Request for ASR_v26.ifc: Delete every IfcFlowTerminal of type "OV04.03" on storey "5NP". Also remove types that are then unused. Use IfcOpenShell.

First a look at what the model holds.

```python
import ifcopenshell
import ifcopenshell.util.element

model = ifcopenshell.open("ASR_v26.ifc")
print(model.schema)
storey = next(s for s in model.by_type("IfcBuildingStorey") if s.Name == "5NP")
terminals = [e for e in ifcopenshell.util.element.get_decomposition(storey) if e.is_a("IfcFlowTerminal")]
seen = {}
for e in terminals:
    element_type = ifcopenshell.util.element.get_type(e)
    name = element_type.Name if element_type not in (None, e) else None
    seen[name] = seen.get(name, 0) + 1
for name, count in sorted(seen.items(), key=str):
    print(count, "x", name)
```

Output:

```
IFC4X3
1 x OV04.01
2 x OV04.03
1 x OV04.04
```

```python
import ifcopenshell
import ifcopenshell.api.root
import ifcopenshell.util.element

model = ifcopenshell.open("ASR_v26.ifc")

storey = next(s for s in model.by_type("IfcBuildingStorey") if s.Name == "5NP")
terminals = [e for e in ifcopenshell.util.element.get_decomposition(storey) if e.is_a("IfcFlowTerminal")]
targets = [e for e in terminals if (t := ifcopenshell.util.element.get_type(e)) not in (None, e) and t.Name == "OV04.03"]
types = {ifcopenshell.util.element.get_type(e) for e in targets} - {None, *targets}

for e in targets:
    ifcopenshell.api.root.remove_product(model, product=e)
print(len(targets), "removed")

unused = [t for t in types if not ifcopenshell.util.element.get_types(t)]
for t in unused:
    ifcopenshell.api.root.remove_product(model, product=t)
print(len(unused), "unused types removed")

model.write("ASR_v26-out.ifc")
```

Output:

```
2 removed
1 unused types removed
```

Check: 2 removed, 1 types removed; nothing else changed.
